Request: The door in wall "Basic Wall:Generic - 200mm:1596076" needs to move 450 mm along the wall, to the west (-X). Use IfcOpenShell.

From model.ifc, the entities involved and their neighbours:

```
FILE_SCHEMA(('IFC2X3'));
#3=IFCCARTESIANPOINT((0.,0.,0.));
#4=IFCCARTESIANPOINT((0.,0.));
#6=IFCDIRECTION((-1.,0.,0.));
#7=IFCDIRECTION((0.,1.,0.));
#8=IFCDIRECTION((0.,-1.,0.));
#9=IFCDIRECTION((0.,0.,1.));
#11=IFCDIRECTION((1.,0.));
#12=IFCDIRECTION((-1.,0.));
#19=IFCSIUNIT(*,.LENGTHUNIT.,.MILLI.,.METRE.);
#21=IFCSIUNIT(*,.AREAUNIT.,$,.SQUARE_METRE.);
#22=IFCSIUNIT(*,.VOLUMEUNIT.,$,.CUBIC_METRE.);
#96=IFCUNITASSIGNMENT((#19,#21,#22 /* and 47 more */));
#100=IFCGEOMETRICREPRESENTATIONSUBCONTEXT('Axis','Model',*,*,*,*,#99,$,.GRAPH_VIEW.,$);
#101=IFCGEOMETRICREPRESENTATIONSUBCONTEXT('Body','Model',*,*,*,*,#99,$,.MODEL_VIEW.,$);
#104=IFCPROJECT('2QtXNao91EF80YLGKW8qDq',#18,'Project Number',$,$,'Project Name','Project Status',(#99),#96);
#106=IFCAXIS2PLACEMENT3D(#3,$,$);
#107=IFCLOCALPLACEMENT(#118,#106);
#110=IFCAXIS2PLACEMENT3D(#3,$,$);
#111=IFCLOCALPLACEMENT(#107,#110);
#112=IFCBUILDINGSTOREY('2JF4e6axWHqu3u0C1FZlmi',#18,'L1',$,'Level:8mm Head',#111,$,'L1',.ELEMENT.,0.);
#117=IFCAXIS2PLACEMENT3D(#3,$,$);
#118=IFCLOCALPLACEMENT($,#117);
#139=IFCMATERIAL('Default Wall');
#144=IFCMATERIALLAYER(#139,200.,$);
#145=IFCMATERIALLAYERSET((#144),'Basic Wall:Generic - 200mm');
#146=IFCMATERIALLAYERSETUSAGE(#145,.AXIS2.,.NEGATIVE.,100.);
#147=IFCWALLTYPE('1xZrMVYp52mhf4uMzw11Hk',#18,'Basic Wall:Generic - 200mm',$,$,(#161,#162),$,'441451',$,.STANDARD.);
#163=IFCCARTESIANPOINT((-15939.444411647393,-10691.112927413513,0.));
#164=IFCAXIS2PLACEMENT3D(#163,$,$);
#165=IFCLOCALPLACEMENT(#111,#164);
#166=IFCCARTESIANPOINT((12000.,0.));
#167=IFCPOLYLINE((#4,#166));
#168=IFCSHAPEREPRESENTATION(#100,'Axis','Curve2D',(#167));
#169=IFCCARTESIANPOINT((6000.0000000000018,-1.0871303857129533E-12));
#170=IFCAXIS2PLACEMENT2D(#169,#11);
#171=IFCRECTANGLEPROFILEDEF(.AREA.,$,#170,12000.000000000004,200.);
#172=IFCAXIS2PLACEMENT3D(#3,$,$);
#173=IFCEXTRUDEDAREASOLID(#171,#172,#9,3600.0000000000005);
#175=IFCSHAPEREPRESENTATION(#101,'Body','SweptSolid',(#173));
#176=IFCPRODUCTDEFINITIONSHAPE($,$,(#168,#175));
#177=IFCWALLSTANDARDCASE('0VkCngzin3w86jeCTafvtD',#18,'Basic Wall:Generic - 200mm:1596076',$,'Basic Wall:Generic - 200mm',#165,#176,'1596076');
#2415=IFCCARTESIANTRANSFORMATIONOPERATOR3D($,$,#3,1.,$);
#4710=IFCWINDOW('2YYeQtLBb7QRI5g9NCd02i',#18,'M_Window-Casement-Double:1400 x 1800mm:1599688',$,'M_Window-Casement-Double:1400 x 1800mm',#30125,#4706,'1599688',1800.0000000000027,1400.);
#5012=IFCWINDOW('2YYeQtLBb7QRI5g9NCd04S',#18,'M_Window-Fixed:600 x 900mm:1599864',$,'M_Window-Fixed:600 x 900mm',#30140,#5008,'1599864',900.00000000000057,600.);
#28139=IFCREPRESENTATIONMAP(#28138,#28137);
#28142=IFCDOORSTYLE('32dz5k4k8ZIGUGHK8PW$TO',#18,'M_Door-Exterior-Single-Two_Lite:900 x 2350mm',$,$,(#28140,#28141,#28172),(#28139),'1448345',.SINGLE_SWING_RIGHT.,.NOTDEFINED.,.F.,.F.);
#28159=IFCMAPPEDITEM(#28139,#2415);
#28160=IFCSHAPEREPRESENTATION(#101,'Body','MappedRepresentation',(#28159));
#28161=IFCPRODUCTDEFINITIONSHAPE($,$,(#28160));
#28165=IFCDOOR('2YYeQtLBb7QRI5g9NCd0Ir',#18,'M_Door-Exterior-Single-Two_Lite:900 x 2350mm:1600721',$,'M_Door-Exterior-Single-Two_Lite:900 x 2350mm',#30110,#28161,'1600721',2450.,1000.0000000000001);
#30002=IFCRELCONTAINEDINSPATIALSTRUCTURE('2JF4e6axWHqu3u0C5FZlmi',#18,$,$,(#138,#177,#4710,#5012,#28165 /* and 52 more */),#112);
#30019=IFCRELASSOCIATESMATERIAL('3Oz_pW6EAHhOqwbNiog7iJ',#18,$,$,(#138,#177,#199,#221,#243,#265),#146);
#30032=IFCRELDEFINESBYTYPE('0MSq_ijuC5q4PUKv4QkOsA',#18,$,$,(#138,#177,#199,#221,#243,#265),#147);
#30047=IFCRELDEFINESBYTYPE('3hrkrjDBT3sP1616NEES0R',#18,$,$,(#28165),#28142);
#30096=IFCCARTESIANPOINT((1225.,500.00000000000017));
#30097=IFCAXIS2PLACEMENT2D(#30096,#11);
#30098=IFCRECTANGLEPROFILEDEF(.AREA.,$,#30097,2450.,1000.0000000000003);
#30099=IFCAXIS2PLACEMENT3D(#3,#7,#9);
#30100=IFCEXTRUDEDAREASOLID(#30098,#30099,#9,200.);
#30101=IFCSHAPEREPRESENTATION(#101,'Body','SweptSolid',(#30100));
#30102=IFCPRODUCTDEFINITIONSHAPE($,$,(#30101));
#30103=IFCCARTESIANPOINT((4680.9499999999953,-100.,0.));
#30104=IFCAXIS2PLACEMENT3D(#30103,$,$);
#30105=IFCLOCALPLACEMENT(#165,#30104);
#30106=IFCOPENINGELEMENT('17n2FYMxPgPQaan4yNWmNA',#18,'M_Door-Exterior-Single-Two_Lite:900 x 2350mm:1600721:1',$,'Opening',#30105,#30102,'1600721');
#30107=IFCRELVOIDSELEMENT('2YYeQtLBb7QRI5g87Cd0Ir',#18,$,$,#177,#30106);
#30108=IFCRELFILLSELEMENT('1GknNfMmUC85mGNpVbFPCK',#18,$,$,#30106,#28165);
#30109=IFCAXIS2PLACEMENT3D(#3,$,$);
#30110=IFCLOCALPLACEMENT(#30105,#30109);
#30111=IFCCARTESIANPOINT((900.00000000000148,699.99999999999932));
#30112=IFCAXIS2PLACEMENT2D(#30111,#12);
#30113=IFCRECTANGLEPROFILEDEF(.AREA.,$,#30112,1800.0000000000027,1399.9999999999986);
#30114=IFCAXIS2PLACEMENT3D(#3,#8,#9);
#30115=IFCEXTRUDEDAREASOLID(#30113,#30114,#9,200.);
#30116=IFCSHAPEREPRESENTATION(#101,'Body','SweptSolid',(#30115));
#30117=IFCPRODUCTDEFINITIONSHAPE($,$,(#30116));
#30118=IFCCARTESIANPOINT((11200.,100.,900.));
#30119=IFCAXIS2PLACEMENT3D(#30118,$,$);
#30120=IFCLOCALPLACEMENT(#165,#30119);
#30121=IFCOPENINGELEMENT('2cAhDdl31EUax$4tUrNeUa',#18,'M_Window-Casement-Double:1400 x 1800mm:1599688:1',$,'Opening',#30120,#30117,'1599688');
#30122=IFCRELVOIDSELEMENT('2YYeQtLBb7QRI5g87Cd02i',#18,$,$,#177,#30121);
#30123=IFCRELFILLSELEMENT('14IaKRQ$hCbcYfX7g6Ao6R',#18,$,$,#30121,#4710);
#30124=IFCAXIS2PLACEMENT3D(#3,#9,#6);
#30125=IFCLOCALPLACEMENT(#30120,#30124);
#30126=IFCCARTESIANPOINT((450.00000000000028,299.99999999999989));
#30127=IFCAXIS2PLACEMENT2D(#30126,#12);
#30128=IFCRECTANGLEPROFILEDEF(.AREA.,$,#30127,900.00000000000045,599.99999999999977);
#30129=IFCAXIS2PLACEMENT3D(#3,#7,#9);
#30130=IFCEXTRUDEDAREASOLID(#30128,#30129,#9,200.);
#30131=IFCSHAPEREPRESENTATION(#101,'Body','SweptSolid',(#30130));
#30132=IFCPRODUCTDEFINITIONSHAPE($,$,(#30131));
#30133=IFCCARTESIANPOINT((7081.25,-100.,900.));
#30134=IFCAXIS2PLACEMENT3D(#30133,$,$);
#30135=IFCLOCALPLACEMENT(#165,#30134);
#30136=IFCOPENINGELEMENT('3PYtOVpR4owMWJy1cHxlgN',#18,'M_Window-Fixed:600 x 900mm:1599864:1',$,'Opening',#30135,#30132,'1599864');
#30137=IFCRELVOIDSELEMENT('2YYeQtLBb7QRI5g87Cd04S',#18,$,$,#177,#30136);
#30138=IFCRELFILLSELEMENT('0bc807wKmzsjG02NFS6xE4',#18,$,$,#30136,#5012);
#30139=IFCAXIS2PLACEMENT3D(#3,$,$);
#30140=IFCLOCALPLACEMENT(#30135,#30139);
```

```python
import ifcopenshell
import ifcopenshell.api.geometry
import ifcopenshell.util.placement

model = ifcopenshell.open("model.ifc")

door = model.by_guid("2YYeQtLBb7QRI5g9NCd0Ir")
opening = door.FillsVoids[0].RelatingOpeningElement
wall = opening.VoidsElements[0].RelatingBuildingElement

wall_matrix = ifcopenshell.util.placement.get_local_placement(wall.ObjectPlacement)
shift = wall_matrix[:3, 0] * -450.0
before = ifcopenshell.util.placement.get_local_placement(door.ObjectPlacement)[:3, 3].copy()

# The door is placed relative to its opening, so it follows when the opening moves.
matrix = ifcopenshell.util.placement.get_local_placement(opening.ObjectPlacement)
matrix[:3, 3] += shift
ifcopenshell.api.geometry.edit_object_placement(
    model, product=opening, matrix=matrix, is_si=False, should_transform_children=True
)

after = ifcopenshell.util.placement.get_local_placement(door.ObjectPlacement)[:3, 3]
print("door moved by", (after - before).round(3) + 0.0)

model.write("model_updated.ifc")
```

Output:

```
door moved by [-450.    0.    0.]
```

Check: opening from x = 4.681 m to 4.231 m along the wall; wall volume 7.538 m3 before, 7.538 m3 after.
